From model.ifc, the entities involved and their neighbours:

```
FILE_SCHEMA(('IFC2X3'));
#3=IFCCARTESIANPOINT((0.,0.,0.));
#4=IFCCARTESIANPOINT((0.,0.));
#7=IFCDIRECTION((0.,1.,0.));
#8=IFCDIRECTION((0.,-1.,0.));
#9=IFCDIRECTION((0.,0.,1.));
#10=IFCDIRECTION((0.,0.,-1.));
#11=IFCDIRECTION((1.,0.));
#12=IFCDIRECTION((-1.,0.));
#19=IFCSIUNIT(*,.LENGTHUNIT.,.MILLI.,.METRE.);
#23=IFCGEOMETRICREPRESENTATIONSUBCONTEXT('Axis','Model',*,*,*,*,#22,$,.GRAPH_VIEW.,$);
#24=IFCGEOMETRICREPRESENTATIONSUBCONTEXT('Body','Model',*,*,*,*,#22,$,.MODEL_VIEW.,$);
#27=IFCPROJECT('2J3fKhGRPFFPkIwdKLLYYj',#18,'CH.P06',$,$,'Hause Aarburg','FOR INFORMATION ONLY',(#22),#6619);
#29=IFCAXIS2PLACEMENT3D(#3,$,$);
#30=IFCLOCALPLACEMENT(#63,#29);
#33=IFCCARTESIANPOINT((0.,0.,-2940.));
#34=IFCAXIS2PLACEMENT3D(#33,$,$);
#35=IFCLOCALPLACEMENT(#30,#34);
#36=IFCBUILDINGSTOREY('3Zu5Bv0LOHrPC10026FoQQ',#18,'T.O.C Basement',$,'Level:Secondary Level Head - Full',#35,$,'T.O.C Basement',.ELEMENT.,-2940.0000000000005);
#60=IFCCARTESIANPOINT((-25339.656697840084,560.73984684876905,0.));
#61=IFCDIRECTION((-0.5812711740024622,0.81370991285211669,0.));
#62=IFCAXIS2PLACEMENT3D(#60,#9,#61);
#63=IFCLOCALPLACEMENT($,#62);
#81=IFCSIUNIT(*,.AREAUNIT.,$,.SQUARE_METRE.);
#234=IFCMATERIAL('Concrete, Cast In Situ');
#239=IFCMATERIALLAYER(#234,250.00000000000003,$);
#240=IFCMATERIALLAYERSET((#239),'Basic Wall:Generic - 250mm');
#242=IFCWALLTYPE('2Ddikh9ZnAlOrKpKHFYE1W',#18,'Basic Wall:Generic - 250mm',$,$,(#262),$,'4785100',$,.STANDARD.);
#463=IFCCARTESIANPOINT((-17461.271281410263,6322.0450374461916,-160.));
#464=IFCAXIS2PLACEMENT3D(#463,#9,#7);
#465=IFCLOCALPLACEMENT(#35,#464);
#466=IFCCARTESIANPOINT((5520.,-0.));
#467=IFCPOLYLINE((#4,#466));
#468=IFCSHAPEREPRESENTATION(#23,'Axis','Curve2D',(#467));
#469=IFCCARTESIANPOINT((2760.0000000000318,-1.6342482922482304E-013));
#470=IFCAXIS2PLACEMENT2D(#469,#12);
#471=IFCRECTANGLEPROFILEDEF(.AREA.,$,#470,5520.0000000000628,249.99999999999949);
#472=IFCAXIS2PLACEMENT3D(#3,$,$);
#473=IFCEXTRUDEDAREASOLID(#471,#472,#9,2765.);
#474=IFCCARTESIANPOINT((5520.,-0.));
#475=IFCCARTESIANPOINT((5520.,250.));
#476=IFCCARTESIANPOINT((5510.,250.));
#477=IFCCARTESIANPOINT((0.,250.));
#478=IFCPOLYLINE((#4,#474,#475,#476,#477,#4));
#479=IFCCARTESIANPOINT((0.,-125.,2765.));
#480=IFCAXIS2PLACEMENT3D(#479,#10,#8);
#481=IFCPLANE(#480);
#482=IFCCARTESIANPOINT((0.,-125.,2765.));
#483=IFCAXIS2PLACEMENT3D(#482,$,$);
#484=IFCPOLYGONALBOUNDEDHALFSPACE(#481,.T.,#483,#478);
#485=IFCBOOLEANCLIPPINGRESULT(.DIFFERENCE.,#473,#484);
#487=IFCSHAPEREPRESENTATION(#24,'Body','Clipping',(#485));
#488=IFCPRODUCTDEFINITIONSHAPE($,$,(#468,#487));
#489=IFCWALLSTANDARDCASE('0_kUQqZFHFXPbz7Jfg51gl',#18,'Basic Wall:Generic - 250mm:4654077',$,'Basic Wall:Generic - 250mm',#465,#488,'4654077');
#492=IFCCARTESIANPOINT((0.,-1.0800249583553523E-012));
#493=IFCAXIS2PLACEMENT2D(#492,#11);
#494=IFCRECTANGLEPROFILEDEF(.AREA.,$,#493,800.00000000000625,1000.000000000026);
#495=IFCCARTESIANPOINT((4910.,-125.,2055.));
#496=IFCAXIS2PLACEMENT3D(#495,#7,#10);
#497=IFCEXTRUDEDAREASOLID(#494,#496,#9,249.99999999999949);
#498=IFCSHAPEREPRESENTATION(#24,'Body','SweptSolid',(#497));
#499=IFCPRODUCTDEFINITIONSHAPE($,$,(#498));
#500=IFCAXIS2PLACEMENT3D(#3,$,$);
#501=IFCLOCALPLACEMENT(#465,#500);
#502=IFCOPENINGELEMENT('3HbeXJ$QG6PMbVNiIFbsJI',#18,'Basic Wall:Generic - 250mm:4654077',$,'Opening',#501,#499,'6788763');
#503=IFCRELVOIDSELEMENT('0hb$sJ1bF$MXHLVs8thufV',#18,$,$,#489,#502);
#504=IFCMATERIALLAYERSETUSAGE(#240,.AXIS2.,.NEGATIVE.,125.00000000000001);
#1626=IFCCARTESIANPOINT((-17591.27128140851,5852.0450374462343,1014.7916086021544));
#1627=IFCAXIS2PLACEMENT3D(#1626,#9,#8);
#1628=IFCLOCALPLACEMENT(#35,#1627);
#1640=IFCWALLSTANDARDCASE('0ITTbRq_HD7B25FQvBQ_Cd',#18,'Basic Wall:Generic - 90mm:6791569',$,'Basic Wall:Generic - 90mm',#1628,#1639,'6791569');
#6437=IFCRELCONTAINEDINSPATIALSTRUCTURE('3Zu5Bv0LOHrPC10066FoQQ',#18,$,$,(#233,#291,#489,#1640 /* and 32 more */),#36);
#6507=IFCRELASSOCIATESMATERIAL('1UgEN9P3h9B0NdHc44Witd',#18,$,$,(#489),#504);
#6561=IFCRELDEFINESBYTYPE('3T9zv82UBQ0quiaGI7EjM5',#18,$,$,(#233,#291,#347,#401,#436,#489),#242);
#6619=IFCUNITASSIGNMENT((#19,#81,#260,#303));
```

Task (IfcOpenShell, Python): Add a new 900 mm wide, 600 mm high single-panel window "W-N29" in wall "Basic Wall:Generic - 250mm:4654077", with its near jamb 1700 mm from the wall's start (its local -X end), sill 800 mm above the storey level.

```python
import numpy as np
import ifcopenshell
import ifcopenshell.api.feature
import ifcopenshell.api.geometry
import ifcopenshell.api.root
import ifcopenshell.api.spatial
import ifcopenshell.api.type
import ifcopenshell.geom
import ifcopenshell.util.element
import ifcopenshell.util.placement
import ifcopenshell.util.representation
import ifcopenshell.util.shape
import ifcopenshell.util.unit

model = ifcopenshell.open("model.ifc")
unit_scale = ifcopenshell.util.unit.calculate_unit_scale(model)
settings = ifcopenshell.geom.settings()


def volume(element):
    """Net volume in cubic metres, openings subtracted."""
    shape = ifcopenshell.geom.create_shape(settings, element)
    return ifcopenshell.util.shape.get_volume(shape.geometry)


wall = model.by_guid("0_kUQqZFHFXPbz7Jfg51gl")
storey = ifcopenshell.util.element.get_container(wall, ifc_class="IfcBuildingStorey")
context = ifcopenshell.util.representation.get_context(model, "Model", "Body", "MODEL_VIEW")
before = volume(wall)

width, height, from_end, sill = 0.9, 0.6, 1.7, 0.8  # metres

# The wall runs along its own X axis, and the end named is its -X end.
wall_shape = ifcopenshell.geom.create_shape(settings, wall)
x, y, z = ifcopenshell.util.shape.get_vertices(wall_shape.geometry).T
start = x.min() + from_end
face, thickness = float(y.min()), float(y.max() - y.min())
wall_matrix = ifcopenshell.util.placement.get_local_placement(wall.ObjectPlacement)
level = ifcopenshell.util.placement.get_local_placement(storey.ObjectPlacement)[2, 3]


def in_wall(x, y):
    """Placement at x, y metres in the wall's axes, at sill height."""
    matrix = wall_matrix.copy()
    matrix[:, 3] = wall_matrix @ np.array([x / unit_scale, y / unit_scale, 0.0, 1.0])
    matrix[2, 3] = level + sill / unit_scale
    return matrix


# Opening: a box that overshoots both wall faces by 50 mm.
opening = ifcopenshell.api.root.create_entity(model, ifc_class="IfcOpeningElement")
box = ifcopenshell.api.geometry.add_wall_representation(
    model, context=context, length=width, height=height, thickness=thickness + 0.1
)
ifcopenshell.api.geometry.assign_representation(model, product=opening, representation=box)
ifcopenshell.api.geometry.edit_object_placement(model, product=opening, matrix=in_wall(start, face - 0.05), is_si=False)
ifcopenshell.api.feature.add_feature(model, feature=opening, element=wall)

window = ifcopenshell.api.root.create_entity(model, ifc_class="IfcWindow", name="W-N29")
window.OverallWidth, window.OverallHeight = width / unit_scale, height / unit_scale
body = ifcopenshell.api.geometry.add_window_representation(
    model,
    context=context,
    overall_width=window.OverallWidth,
    overall_height=window.OverallHeight,
    partition_type="SINGLE_PANEL",
)
ifcopenshell.api.geometry.assign_representation(model, product=window, representation=body)
ifcopenshell.api.spatial.assign_container(model, products=[window], relating_structure=storey)
fills = ifcopenshell.api.feature.add_filling(model, opening=opening, element=window)
fills.OwnerHistory = window.OwnerHistory  # required in IFC2X3

# IFC2X3 keeps the operation on the window style.
style = ifcopenshell.api.root.create_entity(model, ifc_class="IfcWindowStyle", name="W-N29")
style.OperationType, style.ConstructionType = "SINGLE_PANEL", "NOTDEFINED"
style.ParameterTakesPrecedence = style.Sizeable = False
ifcopenshell.api.type.assign_type(model, related_objects=[window], relating_type=style)

# Centre the window in the wall's thickness.
ifcopenshell.api.geometry.edit_object_placement(model, product=window, matrix=in_wall(start, face), is_si=False)
window_shape = ifcopenshell.geom.create_shape(settings, window)
depth = ifcopenshell.util.shape.get_vertices(window_shape.geometry)[:, 1]
offset = face + thickness / 2 - (depth.min() + depth.max()) / 2
ifcopenshell.api.geometry.edit_object_placement(model, product=window, matrix=in_wall(start, offset), is_si=False)

after = volume(wall)

print(f"wall volume {before:.3f} -> {after:.3f} m3")

model.write("model-out.ifc")
```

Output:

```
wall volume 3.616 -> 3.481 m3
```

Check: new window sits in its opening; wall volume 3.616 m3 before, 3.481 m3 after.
